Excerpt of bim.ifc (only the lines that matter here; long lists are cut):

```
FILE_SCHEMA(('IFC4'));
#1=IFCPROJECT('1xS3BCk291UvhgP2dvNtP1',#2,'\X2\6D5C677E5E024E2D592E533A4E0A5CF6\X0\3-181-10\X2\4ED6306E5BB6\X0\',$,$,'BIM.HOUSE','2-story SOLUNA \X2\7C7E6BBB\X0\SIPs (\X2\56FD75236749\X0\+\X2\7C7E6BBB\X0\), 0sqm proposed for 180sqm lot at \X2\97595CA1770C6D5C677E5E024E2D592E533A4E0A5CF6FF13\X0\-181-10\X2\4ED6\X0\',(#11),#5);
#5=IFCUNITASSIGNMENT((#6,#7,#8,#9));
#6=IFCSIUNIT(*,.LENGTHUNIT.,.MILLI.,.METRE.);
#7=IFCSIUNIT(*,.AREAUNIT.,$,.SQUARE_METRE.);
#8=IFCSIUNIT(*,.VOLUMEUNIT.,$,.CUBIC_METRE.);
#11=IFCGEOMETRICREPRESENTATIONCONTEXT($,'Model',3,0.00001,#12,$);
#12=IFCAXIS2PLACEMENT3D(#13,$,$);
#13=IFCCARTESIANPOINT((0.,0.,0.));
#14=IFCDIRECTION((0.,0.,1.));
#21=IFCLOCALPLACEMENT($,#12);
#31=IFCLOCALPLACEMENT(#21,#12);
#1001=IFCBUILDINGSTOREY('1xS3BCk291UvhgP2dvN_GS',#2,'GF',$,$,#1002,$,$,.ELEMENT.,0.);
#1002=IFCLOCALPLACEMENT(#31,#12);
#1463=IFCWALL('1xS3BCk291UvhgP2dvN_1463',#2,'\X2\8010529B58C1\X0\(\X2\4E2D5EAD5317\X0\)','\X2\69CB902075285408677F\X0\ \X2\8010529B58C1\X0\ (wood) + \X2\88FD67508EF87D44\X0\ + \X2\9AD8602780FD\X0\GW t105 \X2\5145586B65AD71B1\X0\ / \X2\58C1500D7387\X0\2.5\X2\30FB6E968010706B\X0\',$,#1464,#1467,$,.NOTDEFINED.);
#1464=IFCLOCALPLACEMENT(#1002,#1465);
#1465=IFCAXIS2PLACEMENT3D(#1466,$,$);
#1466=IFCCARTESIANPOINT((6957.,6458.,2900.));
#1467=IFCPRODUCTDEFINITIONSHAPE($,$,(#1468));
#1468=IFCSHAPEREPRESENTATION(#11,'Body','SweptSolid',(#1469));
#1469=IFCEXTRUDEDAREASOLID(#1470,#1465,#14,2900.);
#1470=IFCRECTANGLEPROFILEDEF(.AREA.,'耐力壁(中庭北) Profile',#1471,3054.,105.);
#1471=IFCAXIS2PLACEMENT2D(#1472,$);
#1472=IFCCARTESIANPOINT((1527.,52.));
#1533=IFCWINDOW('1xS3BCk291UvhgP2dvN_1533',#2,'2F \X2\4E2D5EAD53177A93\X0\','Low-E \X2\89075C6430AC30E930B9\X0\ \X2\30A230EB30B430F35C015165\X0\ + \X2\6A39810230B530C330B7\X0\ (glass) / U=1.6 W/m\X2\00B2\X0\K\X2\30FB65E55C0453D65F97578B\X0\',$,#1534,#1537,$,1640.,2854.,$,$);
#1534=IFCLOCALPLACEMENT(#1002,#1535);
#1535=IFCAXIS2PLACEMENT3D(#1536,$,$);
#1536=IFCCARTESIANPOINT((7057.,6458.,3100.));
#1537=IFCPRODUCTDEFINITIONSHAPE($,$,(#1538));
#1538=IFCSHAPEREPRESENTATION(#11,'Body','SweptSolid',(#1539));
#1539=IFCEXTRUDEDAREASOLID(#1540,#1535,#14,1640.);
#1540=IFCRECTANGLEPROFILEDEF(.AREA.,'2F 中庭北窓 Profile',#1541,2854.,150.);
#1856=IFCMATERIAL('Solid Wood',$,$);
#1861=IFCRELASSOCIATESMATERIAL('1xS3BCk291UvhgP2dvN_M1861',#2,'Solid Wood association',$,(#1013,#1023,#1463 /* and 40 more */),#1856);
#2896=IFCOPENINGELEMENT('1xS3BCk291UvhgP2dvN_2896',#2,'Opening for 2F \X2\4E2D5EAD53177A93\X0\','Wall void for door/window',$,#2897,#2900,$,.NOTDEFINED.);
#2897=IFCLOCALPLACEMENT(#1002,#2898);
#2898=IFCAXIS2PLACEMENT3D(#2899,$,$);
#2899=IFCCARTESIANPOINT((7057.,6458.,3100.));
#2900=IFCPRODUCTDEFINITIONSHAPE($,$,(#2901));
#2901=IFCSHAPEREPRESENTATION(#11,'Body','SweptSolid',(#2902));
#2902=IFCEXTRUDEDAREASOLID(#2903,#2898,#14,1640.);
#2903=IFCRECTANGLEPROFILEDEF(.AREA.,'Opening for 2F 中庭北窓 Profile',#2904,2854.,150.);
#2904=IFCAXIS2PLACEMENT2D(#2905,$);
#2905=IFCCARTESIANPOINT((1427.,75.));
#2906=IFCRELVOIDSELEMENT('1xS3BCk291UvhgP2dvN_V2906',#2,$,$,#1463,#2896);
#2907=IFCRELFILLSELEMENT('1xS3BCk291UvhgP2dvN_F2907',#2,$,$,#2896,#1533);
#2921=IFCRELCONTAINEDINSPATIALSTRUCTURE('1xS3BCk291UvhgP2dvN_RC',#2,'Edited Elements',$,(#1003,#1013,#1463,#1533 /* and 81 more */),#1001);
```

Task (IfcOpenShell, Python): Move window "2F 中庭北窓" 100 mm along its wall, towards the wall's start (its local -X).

```python
import ifcopenshell
import ifcopenshell.api.geometry
import ifcopenshell.util.placement
import ifcopenshell.util.unit

model = ifcopenshell.open("bim.ifc")
unit_scale = ifcopenshell.util.unit.calculate_unit_scale(model)

window = model.by_guid("1xS3BCk291UvhgP2dvN_1533")
opening = window.FillsVoids[0].RelatingOpeningElement
wall = opening.VoidsElements[0].RelatingBuildingElement

wall_matrix = ifcopenshell.util.placement.get_local_placement(wall.ObjectPlacement)
shift = wall_matrix[:3, 0] * -0.1 / unit_scale
before = ifcopenshell.util.placement.get_local_placement(window.ObjectPlacement)[:3, 3].copy()

# The window is not placed relative to its opening, so move both.
for product in (opening, window):
    matrix = ifcopenshell.util.placement.get_local_placement(product.ObjectPlacement)
    matrix[:3, 3] += shift
    ifcopenshell.api.geometry.edit_object_placement(model, product=product, matrix=matrix, is_si=False)

after = ifcopenshell.util.placement.get_local_placement(window.ObjectPlacement)[:3, 3]
print("window moved by", (after - before).round(3) + 0.0)

model.write("bim_edited.ifc")
```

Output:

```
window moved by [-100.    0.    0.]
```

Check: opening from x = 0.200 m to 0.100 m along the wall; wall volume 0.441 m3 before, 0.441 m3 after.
